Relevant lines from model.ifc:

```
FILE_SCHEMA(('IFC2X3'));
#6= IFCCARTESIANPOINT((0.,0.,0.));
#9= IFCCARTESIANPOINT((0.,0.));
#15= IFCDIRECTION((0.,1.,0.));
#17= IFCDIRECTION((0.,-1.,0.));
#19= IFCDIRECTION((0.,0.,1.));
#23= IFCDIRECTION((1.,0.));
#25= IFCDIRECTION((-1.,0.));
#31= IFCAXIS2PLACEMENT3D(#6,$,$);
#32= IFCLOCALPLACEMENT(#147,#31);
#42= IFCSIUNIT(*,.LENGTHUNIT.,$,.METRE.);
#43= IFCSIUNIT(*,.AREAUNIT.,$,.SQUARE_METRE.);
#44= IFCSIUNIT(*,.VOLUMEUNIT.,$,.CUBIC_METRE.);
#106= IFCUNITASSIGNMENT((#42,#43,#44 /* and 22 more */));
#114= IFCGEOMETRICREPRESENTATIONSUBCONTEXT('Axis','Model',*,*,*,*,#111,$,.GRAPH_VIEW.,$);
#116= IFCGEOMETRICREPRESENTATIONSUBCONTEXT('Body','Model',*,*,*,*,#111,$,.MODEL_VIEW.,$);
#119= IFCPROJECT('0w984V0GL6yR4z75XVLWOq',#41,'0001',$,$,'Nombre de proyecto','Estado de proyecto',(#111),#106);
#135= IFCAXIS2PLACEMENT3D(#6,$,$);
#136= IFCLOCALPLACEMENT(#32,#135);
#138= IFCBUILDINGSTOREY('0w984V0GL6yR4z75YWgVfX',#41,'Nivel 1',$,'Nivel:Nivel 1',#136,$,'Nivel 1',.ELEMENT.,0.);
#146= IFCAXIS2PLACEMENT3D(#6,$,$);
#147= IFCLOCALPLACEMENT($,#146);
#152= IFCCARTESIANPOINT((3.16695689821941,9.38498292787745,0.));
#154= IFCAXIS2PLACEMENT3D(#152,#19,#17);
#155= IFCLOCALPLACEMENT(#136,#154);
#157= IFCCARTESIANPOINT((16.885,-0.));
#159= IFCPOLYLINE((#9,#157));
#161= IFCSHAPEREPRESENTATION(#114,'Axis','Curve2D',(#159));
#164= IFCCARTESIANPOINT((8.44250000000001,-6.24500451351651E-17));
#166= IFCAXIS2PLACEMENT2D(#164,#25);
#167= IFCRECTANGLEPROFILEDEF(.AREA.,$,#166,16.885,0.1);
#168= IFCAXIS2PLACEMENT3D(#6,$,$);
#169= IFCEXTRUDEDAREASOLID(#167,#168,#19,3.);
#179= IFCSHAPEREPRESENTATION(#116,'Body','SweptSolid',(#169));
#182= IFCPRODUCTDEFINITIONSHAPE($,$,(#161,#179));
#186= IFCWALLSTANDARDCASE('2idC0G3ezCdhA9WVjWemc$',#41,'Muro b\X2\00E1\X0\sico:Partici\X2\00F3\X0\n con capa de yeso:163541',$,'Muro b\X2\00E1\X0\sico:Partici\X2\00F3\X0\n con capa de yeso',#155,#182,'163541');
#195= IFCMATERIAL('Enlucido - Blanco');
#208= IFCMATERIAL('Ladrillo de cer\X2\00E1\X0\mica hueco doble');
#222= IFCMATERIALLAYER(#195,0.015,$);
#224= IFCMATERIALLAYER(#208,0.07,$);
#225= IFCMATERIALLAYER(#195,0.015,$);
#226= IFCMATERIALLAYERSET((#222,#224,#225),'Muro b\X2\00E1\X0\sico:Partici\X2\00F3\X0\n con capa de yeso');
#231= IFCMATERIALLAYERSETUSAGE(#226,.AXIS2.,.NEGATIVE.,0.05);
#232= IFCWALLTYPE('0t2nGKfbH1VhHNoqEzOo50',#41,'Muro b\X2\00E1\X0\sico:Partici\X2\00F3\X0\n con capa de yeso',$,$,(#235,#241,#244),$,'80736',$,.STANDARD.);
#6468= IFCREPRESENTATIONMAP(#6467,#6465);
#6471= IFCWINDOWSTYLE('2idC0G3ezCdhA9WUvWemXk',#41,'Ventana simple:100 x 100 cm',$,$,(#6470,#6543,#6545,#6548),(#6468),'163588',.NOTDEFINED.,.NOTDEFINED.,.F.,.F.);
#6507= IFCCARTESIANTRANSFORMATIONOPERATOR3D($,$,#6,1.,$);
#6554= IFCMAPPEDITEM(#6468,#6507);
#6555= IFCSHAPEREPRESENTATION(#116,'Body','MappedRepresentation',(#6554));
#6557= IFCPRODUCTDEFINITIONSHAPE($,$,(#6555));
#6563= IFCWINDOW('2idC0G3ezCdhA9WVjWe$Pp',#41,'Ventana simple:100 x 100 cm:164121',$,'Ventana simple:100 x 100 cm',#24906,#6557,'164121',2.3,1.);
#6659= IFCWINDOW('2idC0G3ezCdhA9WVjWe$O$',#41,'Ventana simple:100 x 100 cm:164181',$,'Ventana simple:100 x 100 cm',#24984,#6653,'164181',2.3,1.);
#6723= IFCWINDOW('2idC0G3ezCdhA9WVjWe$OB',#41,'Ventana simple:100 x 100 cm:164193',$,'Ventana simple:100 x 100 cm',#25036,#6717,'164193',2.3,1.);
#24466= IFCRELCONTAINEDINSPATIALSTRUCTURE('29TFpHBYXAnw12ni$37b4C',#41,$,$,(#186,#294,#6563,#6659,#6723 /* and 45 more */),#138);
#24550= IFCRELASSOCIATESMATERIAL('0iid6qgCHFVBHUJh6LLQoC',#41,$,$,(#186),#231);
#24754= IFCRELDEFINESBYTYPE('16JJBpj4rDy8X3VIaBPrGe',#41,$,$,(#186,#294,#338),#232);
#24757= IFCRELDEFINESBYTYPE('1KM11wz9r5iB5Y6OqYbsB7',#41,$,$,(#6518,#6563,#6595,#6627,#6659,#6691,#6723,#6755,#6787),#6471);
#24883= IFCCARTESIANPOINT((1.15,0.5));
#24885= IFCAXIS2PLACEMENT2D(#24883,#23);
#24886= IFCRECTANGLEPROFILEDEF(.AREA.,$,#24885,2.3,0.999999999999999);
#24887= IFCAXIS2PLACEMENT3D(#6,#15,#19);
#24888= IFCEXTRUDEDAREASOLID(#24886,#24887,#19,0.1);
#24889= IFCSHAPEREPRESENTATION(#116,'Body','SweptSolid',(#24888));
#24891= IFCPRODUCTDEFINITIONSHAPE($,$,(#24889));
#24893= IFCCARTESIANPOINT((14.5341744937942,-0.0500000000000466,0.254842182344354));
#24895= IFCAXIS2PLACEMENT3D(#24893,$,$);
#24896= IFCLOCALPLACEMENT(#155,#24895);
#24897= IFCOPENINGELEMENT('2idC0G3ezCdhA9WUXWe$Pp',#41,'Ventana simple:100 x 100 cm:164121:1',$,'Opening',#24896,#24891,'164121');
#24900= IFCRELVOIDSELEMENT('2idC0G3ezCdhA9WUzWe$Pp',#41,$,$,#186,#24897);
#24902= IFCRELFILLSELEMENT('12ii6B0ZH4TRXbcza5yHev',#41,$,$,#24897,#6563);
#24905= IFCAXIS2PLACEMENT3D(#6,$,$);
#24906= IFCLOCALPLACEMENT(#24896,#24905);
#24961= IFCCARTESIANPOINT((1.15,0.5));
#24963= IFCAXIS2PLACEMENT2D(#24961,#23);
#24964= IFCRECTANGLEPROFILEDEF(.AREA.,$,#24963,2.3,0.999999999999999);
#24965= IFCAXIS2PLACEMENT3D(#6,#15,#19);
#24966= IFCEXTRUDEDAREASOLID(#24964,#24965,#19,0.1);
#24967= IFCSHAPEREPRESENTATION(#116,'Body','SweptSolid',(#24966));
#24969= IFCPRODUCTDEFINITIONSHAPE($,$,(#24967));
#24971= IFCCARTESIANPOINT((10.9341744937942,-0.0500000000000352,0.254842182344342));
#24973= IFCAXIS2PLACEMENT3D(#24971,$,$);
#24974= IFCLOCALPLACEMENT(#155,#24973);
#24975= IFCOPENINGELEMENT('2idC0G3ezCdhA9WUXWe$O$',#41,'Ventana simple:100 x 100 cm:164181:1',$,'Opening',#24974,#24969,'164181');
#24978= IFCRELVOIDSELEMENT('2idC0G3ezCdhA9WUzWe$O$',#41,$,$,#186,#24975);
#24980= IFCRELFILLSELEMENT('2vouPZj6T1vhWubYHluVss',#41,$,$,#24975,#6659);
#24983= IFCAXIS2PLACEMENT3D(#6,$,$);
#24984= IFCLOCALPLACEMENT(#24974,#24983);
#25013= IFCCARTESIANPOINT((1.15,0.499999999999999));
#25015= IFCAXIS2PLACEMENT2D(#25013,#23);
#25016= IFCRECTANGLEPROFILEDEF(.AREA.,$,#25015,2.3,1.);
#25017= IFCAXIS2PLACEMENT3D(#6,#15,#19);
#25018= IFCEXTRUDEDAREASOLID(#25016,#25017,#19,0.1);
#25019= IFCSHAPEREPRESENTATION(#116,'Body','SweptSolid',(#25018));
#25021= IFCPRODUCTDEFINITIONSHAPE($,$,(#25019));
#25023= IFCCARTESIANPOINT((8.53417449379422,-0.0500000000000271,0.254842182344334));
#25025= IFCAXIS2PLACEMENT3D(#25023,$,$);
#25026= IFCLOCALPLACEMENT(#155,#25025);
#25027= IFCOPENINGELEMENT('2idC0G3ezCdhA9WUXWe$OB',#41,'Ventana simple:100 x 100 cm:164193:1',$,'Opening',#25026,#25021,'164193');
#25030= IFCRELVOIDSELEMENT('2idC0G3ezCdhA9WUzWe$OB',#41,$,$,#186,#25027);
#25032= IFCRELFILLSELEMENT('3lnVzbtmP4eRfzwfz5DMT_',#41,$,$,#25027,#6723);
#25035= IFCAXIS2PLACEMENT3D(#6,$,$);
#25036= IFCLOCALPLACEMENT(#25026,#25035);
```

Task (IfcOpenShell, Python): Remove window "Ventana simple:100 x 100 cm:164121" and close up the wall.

```python
import ifcopenshell
import ifcopenshell.api.feature
import ifcopenshell.api.root
import ifcopenshell.geom
import ifcopenshell.util.shape

model = ifcopenshell.open("model.ifc")
settings = ifcopenshell.geom.settings()


def volume(element):
    """Net volume in cubic metres, openings subtracted."""
    shape = ifcopenshell.geom.create_shape(settings, element)
    return ifcopenshell.util.shape.get_volume(shape.geometry)


window = model.by_guid("2idC0G3ezCdhA9WVjWe$Pp")
opening = window.FillsVoids[0].RelatingOpeningElement
wall = opening.VoidsElements[0].RelatingBuildingElement
before = volume(wall)

ifcopenshell.api.root.remove_product(model, product=window)
ifcopenshell.api.feature.remove_feature(model, feature=opening)

after = volume(wall)

print(f"wall volume {before:.3f} -> {after:.3f} m3")

model.write("model-out.ifc")
```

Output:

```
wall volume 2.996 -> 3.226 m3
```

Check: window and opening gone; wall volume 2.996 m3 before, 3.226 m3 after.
